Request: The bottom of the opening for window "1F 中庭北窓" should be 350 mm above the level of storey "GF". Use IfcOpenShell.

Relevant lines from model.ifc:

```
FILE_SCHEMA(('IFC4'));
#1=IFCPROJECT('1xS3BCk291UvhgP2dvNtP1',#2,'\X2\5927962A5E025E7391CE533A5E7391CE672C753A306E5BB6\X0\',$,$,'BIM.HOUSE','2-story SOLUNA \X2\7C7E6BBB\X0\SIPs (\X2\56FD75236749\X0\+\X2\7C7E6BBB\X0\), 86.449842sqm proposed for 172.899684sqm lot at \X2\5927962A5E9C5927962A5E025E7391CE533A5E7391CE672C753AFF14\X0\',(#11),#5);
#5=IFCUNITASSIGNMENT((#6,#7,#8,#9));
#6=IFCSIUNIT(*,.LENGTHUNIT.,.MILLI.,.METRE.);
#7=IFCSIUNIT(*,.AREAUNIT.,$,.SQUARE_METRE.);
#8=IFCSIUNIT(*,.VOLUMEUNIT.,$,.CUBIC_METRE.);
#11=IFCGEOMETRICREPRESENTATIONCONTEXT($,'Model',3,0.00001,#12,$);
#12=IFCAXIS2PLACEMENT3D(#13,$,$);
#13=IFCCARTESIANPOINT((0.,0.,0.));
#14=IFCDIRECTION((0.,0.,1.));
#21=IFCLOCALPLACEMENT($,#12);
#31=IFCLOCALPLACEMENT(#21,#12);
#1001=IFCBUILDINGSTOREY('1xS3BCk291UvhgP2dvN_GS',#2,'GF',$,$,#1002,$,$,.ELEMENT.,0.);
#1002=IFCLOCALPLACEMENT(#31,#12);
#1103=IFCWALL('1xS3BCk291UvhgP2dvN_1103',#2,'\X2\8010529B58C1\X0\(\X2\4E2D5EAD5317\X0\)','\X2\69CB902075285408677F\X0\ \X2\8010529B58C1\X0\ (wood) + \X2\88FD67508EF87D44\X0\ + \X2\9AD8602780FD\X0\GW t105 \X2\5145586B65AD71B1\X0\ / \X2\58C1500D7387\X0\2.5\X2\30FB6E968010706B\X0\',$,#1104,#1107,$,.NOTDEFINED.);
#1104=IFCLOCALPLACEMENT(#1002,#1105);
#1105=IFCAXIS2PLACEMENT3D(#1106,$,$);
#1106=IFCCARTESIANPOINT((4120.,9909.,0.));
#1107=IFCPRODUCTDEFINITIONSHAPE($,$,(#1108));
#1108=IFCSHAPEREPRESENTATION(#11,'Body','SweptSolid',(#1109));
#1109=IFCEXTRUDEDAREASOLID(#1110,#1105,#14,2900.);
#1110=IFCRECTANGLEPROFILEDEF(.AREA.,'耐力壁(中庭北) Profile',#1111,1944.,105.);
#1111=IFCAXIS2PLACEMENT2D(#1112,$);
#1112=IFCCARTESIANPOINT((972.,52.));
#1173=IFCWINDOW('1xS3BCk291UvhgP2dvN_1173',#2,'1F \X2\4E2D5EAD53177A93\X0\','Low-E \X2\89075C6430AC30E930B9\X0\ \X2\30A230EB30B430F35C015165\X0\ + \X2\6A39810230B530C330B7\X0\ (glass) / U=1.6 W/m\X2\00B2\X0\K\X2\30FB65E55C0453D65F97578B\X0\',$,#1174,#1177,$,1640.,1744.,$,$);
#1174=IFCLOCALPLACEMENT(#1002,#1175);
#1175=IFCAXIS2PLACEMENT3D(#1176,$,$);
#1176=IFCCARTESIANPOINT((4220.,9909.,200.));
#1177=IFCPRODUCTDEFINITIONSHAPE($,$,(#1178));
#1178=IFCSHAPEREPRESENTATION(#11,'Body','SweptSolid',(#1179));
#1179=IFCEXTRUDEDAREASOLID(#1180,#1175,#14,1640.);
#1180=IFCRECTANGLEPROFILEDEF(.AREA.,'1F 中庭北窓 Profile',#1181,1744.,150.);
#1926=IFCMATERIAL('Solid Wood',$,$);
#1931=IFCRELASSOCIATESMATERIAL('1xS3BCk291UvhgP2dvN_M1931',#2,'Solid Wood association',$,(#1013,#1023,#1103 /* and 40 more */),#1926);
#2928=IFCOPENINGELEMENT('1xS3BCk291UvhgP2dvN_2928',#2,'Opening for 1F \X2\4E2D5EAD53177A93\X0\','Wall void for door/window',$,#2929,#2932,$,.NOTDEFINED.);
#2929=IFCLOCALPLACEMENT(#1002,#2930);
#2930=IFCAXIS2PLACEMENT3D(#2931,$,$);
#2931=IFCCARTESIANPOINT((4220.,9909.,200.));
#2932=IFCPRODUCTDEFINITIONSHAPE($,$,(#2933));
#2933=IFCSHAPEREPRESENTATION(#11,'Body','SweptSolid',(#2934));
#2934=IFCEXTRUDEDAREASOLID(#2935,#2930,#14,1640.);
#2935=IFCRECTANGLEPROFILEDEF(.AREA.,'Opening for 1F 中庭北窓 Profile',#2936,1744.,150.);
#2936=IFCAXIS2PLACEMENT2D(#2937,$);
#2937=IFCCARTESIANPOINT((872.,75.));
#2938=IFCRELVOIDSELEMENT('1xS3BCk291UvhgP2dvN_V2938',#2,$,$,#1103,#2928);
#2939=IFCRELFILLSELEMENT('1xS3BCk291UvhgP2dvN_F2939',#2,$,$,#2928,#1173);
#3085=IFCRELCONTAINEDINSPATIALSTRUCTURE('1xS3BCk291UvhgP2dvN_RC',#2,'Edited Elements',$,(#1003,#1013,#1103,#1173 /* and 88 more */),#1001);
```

```python
import numpy as np
import ifcopenshell
import ifcopenshell.api.geometry
import ifcopenshell.geom
import ifcopenshell.util.element
import ifcopenshell.util.placement
import ifcopenshell.util.shape
import ifcopenshell.util.unit

model = ifcopenshell.open("model.ifc")
unit_scale = ifcopenshell.util.unit.calculate_unit_scale(model)

window = model.by_guid("1xS3BCk291UvhgP2dvN_1173")
opening = window.FillsVoids[0].RelatingOpeningElement
storey = ifcopenshell.util.element.get_container(window, ifc_class="IfcBuildingStorey")
level = ifcopenshell.util.placement.get_local_placement(storey.ObjectPlacement)[2, 3]

# The opening's origin need not be at the sill, so measure its lowest point.
shape = ifcopenshell.geom.create_shape(ifcopenshell.geom.settings(), opening)
bottom = ifcopenshell.util.shape.get_shape_bottom_elevation(shape, shape.geometry) / unit_scale
dz = level + 350.0 - bottom

shift = np.array([0.0, 0.0, dz])
# The window is not placed relative to its opening, so move both.
for product in (opening, window):
    matrix = ifcopenshell.util.placement.get_local_placement(product.ObjectPlacement)
    matrix[:3, 3] += shift
    ifcopenshell.api.geometry.edit_object_placement(model, product=product, matrix=matrix, is_si=False)

print(f"moved by {dz * unit_scale:+.3f} m")

model.write("model_updated.ifc")
```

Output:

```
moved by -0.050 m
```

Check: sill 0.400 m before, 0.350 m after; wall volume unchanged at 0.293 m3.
